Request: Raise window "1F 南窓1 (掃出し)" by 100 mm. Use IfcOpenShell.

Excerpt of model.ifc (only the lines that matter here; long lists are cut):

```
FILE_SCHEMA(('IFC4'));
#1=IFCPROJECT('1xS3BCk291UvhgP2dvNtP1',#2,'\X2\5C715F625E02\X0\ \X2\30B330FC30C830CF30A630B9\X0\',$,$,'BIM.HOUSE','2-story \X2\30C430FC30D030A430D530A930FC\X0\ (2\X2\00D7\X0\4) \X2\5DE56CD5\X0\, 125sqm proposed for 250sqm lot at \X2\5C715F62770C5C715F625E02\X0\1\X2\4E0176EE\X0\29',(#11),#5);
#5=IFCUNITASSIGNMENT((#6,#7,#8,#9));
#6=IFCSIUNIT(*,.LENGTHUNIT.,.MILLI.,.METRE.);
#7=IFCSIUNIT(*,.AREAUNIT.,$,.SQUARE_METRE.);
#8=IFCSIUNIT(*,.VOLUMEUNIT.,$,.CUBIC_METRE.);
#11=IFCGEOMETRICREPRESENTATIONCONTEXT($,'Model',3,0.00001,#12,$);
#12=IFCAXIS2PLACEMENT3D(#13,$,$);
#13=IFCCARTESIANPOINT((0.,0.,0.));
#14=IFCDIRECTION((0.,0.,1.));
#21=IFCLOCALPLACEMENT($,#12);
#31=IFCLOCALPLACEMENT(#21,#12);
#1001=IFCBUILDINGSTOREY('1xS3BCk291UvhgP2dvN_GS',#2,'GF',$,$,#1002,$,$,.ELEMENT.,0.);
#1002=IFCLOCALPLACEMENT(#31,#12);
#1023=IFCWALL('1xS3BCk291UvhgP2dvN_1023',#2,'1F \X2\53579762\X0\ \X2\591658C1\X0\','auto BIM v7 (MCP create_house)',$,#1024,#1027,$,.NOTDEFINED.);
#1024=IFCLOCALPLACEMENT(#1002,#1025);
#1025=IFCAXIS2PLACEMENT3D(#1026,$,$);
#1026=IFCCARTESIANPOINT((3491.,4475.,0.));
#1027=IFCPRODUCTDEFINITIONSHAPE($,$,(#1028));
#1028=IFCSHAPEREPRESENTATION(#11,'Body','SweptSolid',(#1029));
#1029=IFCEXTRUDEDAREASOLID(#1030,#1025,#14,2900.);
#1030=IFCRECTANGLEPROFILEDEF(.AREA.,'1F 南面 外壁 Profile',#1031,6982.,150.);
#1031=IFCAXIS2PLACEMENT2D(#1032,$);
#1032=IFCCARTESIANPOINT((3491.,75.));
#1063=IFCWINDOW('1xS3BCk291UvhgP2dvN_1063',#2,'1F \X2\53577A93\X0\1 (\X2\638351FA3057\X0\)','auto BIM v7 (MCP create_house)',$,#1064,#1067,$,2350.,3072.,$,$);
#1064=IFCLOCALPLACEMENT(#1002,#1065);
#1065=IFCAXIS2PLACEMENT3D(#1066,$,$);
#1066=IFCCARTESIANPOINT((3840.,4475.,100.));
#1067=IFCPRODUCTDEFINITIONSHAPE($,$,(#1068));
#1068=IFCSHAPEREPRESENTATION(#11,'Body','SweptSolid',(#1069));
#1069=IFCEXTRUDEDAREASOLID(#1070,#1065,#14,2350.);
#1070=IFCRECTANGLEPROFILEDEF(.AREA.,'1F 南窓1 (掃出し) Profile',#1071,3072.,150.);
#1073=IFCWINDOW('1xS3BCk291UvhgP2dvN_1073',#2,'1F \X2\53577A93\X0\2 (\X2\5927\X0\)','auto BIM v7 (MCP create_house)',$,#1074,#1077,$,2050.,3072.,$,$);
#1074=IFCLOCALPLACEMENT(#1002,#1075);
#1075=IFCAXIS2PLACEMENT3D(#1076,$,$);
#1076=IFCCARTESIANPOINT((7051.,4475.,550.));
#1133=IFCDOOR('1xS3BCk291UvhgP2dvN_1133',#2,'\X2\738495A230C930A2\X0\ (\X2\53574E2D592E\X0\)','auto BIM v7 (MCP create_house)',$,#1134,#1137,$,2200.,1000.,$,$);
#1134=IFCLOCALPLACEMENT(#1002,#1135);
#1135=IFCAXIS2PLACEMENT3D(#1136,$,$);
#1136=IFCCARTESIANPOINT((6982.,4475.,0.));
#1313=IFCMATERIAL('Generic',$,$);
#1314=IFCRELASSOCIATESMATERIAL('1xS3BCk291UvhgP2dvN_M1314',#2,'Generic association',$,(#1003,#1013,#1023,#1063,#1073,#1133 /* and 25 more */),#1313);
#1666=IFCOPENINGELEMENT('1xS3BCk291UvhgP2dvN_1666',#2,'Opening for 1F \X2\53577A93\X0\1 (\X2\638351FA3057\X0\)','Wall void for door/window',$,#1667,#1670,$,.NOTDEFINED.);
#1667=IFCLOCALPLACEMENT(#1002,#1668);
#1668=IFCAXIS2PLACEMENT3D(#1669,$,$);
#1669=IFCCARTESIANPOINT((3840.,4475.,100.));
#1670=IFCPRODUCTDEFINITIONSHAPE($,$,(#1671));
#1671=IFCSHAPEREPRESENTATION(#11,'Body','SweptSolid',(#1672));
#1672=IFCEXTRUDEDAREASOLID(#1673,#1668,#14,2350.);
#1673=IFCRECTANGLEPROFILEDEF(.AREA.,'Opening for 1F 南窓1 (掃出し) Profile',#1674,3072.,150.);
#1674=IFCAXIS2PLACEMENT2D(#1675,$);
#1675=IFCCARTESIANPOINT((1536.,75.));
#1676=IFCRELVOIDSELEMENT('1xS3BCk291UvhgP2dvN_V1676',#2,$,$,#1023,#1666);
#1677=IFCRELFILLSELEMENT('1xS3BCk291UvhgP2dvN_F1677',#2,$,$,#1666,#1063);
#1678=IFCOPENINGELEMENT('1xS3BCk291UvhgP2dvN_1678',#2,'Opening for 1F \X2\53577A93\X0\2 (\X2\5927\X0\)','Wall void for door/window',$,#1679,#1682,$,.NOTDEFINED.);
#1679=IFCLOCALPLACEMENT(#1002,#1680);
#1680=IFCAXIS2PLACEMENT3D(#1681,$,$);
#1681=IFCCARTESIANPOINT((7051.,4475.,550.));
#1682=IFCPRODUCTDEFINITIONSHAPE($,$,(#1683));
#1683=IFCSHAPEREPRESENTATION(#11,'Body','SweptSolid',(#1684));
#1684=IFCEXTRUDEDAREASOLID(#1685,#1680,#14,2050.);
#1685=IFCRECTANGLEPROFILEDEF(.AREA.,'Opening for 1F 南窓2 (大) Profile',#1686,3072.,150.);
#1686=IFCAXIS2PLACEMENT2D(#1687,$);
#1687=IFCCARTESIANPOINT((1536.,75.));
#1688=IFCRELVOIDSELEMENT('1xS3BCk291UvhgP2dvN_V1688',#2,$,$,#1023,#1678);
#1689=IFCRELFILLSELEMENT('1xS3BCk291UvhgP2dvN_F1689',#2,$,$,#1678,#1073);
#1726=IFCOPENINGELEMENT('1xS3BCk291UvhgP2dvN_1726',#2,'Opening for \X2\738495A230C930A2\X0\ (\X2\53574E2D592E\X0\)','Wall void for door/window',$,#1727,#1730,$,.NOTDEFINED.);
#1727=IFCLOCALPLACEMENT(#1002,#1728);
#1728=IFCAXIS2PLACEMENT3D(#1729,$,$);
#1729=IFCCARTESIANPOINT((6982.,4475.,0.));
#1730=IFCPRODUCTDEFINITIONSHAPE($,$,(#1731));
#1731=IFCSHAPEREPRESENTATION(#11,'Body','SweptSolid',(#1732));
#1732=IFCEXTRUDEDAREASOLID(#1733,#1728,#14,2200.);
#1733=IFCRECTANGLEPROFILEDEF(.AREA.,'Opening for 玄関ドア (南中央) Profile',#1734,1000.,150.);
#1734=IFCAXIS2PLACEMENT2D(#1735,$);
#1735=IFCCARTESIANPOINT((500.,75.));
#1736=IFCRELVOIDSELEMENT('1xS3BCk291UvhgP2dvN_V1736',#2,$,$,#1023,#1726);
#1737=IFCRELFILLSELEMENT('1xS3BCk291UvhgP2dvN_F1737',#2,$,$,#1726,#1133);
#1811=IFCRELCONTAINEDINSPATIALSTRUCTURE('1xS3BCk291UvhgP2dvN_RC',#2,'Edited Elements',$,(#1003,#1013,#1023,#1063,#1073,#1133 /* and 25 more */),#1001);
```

```python
import numpy as np
import ifcopenshell
import ifcopenshell.api.geometry
import ifcopenshell.util.placement
import ifcopenshell.util.unit

model = ifcopenshell.open("model.ifc")
unit_scale = ifcopenshell.util.unit.calculate_unit_scale(model)

window = model.by_guid("1xS3BCk291UvhgP2dvN_1063")
opening = window.FillsVoids[0].RelatingOpeningElement
dz = 0.1 / unit_scale

shift = np.array([0.0, 0.0, dz])
# The window is not placed relative to its opening, so move both.
for product in (opening, window):
    matrix = ifcopenshell.util.placement.get_local_placement(product.ObjectPlacement)
    matrix[:3, 3] += shift
    ifcopenshell.api.geometry.edit_object_placement(model, product=product, matrix=matrix, is_si=False)

print(f"moved by {dz * unit_scale:+.3f} m")

model.write("model_updated.ifc")
```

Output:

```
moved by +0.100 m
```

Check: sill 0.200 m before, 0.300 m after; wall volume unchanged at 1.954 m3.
